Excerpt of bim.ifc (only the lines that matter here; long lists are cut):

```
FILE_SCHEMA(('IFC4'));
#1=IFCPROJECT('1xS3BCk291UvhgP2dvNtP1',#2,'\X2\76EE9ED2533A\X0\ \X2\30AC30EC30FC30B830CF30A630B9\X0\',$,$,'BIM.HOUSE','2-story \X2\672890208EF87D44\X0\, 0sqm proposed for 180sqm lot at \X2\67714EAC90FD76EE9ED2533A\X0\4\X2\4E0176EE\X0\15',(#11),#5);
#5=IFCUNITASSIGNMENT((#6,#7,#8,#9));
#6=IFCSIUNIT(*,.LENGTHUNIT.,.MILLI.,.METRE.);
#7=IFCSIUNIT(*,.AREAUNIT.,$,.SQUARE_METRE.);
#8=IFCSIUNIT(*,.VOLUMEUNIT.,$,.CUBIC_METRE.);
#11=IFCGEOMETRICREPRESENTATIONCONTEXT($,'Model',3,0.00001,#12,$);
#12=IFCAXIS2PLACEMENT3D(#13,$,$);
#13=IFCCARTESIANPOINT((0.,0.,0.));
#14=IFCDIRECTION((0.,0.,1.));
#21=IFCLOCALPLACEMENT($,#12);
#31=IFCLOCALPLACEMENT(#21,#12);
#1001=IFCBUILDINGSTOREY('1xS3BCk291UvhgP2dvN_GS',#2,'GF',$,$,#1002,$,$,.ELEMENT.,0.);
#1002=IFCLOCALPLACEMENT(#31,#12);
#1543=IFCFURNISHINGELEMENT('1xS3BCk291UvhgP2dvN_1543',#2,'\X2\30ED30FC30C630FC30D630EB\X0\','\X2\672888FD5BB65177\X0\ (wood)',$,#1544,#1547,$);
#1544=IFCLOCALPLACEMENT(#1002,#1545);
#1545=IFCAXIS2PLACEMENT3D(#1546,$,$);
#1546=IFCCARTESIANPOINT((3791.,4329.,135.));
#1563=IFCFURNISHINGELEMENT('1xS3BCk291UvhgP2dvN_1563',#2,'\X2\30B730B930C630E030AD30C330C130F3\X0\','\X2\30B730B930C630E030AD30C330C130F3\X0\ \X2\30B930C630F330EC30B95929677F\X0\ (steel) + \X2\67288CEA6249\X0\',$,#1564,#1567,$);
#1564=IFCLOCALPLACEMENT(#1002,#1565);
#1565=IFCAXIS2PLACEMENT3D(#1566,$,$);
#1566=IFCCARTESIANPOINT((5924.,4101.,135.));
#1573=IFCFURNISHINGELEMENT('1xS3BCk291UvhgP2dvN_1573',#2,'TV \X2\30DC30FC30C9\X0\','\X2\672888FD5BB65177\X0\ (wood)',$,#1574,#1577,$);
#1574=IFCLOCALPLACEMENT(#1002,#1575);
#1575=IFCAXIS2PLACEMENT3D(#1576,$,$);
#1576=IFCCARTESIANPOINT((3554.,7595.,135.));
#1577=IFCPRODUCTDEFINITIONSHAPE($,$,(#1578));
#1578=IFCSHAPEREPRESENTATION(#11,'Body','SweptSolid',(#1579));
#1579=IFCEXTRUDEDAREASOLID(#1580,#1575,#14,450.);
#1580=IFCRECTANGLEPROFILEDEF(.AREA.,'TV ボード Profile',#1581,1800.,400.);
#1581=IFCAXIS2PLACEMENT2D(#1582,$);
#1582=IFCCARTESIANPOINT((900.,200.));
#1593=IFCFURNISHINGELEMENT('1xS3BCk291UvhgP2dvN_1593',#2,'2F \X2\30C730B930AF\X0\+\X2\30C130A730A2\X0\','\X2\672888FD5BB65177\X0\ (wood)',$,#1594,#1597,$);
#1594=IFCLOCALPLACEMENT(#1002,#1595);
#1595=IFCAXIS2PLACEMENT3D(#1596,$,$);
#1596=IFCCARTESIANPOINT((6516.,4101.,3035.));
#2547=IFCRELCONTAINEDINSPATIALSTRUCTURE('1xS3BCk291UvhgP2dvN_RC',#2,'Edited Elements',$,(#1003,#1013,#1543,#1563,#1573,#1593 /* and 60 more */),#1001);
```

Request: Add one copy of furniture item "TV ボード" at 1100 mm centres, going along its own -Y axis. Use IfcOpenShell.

```python
import ifcopenshell
import ifcopenshell.api.geometry
import ifcopenshell.api.root
import ifcopenshell.util.element
import ifcopenshell.util.placement

model = ifcopenshell.open("bim.ifc")


def reuse_history(source, copy):
    """copy_class also copies each property set's owner history, people and application; keep the originals."""
    for rel in copy.IsDefinedBy:
        if rel.is_a("IfcRelDefinesByProperties") and (history := rel.RelatingPropertyDefinition.OwnerHistory):
            rel.RelatingPropertyDefinition.OwnerHistory = source.OwnerHistory
            ifcopenshell.util.element.remove_deep2(model, history)


source = model.by_id(1573)
base = ifcopenshell.util.placement.get_local_placement(source.ObjectPlacement)
step = -base[:3, 1] * 1100.0

for i in range(1, 2):
    copy = ifcopenshell.api.root.copy_class(model, product=source)
    copy.Representation = ifcopenshell.util.element.copy_deep(
        model, source.Representation, exclude=["IfcGeometricRepresentationContext", "IfcRepresentationMap"]
    )
    reuse_history(source, copy)
    matrix = base.copy()
    matrix[:3, 3] += i * step
    print("added at", matrix[:3, 3].round(3) + 0.0)
    ifcopenshell.api.geometry.edit_object_placement(model, product=copy, matrix=matrix, is_si=False)

model.write("bim_rev.ifc")
```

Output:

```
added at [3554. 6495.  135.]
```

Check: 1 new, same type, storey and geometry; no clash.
